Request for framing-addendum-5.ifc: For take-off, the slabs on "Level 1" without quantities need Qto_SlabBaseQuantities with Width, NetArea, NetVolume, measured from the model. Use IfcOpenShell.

First a look at what the model holds.

```python
import ifcopenshell
import ifcopenshell.util.element
import ifcopenshell.util.unit

model = ifcopenshell.open("framing-addendum-5.ifc")
print(model.schema)
for unit_type in ("LENGTHUNIT", "AREAUNIT", "VOLUMEUNIT"):
    print(unit_type, ifcopenshell.util.unit.calculate_unit_scale(model, unit_type))
storey = next(s for s in model.by_type("IfcBuildingStorey") if s.Name == "Level 1")
slabs = [e for e in ifcopenshell.util.element.get_decomposition(storey) if e.is_a("IfcSlab")]
for e in sorted(slabs, key=lambda e: e.id()):
    print(e.id(), e.is_a(), e.Name, list(ifcopenshell.util.element.get_psets(e, qtos_only=True)), sep=" | ")
```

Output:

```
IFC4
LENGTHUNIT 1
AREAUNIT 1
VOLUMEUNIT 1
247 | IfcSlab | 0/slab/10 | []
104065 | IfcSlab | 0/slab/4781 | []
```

```python
import ifcopenshell
import ifcopenshell.api.pset
import ifcopenshell.geom
import ifcopenshell.util.element
import ifcopenshell.util.shape
import ifcopenshell.util.unit

model = ifcopenshell.open("framing-addendum-5.ifc")
unit_scale = ifcopenshell.util.unit.calculate_unit_scale(model)
area_scale = ifcopenshell.util.unit.calculate_unit_scale(model, "AREAUNIT")
volume_scale = ifcopenshell.util.unit.calculate_unit_scale(model, "VOLUMEUNIT")
settings = ifcopenshell.geom.settings()

storey = next(s for s in model.by_type("IfcBuildingStorey") if s.Name == "Level 1")
slabs = [e for e in ifcopenshell.util.element.get_decomposition(storey) if e.is_a("IfcSlab")]

for e in sorted(slabs, key=lambda e: e.id()):
    if ifcopenshell.util.element.get_psets(e, qtos_only=True, should_inherit=False):
        continue
    # Geometry comes back in metres, in the element's own axes.
    shape = ifcopenshell.geom.create_shape(settings, e)
    values = {
        "Width": ifcopenshell.util.shape.get_z(shape.geometry) / unit_scale,
        "NetArea": ifcopenshell.util.shape.get_footprint_area(shape.geometry) / area_scale,
        "NetVolume": ifcopenshell.util.shape.get_volume(shape.geometry) / volume_scale,
    }
    qto = ifcopenshell.api.pset.add_qto(model, product=e, name="Qto_SlabBaseQuantities")
    ifcopenshell.api.pset.edit_qto(model, qto=qto, properties=values)
    print(e.id(), {k: round(v, 3) for k, v in values.items()})

model.write("framing-addendum-5-out.ifc")
```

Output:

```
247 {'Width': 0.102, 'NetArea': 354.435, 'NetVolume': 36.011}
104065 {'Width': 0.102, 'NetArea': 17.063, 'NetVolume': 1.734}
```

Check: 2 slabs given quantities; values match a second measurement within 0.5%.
